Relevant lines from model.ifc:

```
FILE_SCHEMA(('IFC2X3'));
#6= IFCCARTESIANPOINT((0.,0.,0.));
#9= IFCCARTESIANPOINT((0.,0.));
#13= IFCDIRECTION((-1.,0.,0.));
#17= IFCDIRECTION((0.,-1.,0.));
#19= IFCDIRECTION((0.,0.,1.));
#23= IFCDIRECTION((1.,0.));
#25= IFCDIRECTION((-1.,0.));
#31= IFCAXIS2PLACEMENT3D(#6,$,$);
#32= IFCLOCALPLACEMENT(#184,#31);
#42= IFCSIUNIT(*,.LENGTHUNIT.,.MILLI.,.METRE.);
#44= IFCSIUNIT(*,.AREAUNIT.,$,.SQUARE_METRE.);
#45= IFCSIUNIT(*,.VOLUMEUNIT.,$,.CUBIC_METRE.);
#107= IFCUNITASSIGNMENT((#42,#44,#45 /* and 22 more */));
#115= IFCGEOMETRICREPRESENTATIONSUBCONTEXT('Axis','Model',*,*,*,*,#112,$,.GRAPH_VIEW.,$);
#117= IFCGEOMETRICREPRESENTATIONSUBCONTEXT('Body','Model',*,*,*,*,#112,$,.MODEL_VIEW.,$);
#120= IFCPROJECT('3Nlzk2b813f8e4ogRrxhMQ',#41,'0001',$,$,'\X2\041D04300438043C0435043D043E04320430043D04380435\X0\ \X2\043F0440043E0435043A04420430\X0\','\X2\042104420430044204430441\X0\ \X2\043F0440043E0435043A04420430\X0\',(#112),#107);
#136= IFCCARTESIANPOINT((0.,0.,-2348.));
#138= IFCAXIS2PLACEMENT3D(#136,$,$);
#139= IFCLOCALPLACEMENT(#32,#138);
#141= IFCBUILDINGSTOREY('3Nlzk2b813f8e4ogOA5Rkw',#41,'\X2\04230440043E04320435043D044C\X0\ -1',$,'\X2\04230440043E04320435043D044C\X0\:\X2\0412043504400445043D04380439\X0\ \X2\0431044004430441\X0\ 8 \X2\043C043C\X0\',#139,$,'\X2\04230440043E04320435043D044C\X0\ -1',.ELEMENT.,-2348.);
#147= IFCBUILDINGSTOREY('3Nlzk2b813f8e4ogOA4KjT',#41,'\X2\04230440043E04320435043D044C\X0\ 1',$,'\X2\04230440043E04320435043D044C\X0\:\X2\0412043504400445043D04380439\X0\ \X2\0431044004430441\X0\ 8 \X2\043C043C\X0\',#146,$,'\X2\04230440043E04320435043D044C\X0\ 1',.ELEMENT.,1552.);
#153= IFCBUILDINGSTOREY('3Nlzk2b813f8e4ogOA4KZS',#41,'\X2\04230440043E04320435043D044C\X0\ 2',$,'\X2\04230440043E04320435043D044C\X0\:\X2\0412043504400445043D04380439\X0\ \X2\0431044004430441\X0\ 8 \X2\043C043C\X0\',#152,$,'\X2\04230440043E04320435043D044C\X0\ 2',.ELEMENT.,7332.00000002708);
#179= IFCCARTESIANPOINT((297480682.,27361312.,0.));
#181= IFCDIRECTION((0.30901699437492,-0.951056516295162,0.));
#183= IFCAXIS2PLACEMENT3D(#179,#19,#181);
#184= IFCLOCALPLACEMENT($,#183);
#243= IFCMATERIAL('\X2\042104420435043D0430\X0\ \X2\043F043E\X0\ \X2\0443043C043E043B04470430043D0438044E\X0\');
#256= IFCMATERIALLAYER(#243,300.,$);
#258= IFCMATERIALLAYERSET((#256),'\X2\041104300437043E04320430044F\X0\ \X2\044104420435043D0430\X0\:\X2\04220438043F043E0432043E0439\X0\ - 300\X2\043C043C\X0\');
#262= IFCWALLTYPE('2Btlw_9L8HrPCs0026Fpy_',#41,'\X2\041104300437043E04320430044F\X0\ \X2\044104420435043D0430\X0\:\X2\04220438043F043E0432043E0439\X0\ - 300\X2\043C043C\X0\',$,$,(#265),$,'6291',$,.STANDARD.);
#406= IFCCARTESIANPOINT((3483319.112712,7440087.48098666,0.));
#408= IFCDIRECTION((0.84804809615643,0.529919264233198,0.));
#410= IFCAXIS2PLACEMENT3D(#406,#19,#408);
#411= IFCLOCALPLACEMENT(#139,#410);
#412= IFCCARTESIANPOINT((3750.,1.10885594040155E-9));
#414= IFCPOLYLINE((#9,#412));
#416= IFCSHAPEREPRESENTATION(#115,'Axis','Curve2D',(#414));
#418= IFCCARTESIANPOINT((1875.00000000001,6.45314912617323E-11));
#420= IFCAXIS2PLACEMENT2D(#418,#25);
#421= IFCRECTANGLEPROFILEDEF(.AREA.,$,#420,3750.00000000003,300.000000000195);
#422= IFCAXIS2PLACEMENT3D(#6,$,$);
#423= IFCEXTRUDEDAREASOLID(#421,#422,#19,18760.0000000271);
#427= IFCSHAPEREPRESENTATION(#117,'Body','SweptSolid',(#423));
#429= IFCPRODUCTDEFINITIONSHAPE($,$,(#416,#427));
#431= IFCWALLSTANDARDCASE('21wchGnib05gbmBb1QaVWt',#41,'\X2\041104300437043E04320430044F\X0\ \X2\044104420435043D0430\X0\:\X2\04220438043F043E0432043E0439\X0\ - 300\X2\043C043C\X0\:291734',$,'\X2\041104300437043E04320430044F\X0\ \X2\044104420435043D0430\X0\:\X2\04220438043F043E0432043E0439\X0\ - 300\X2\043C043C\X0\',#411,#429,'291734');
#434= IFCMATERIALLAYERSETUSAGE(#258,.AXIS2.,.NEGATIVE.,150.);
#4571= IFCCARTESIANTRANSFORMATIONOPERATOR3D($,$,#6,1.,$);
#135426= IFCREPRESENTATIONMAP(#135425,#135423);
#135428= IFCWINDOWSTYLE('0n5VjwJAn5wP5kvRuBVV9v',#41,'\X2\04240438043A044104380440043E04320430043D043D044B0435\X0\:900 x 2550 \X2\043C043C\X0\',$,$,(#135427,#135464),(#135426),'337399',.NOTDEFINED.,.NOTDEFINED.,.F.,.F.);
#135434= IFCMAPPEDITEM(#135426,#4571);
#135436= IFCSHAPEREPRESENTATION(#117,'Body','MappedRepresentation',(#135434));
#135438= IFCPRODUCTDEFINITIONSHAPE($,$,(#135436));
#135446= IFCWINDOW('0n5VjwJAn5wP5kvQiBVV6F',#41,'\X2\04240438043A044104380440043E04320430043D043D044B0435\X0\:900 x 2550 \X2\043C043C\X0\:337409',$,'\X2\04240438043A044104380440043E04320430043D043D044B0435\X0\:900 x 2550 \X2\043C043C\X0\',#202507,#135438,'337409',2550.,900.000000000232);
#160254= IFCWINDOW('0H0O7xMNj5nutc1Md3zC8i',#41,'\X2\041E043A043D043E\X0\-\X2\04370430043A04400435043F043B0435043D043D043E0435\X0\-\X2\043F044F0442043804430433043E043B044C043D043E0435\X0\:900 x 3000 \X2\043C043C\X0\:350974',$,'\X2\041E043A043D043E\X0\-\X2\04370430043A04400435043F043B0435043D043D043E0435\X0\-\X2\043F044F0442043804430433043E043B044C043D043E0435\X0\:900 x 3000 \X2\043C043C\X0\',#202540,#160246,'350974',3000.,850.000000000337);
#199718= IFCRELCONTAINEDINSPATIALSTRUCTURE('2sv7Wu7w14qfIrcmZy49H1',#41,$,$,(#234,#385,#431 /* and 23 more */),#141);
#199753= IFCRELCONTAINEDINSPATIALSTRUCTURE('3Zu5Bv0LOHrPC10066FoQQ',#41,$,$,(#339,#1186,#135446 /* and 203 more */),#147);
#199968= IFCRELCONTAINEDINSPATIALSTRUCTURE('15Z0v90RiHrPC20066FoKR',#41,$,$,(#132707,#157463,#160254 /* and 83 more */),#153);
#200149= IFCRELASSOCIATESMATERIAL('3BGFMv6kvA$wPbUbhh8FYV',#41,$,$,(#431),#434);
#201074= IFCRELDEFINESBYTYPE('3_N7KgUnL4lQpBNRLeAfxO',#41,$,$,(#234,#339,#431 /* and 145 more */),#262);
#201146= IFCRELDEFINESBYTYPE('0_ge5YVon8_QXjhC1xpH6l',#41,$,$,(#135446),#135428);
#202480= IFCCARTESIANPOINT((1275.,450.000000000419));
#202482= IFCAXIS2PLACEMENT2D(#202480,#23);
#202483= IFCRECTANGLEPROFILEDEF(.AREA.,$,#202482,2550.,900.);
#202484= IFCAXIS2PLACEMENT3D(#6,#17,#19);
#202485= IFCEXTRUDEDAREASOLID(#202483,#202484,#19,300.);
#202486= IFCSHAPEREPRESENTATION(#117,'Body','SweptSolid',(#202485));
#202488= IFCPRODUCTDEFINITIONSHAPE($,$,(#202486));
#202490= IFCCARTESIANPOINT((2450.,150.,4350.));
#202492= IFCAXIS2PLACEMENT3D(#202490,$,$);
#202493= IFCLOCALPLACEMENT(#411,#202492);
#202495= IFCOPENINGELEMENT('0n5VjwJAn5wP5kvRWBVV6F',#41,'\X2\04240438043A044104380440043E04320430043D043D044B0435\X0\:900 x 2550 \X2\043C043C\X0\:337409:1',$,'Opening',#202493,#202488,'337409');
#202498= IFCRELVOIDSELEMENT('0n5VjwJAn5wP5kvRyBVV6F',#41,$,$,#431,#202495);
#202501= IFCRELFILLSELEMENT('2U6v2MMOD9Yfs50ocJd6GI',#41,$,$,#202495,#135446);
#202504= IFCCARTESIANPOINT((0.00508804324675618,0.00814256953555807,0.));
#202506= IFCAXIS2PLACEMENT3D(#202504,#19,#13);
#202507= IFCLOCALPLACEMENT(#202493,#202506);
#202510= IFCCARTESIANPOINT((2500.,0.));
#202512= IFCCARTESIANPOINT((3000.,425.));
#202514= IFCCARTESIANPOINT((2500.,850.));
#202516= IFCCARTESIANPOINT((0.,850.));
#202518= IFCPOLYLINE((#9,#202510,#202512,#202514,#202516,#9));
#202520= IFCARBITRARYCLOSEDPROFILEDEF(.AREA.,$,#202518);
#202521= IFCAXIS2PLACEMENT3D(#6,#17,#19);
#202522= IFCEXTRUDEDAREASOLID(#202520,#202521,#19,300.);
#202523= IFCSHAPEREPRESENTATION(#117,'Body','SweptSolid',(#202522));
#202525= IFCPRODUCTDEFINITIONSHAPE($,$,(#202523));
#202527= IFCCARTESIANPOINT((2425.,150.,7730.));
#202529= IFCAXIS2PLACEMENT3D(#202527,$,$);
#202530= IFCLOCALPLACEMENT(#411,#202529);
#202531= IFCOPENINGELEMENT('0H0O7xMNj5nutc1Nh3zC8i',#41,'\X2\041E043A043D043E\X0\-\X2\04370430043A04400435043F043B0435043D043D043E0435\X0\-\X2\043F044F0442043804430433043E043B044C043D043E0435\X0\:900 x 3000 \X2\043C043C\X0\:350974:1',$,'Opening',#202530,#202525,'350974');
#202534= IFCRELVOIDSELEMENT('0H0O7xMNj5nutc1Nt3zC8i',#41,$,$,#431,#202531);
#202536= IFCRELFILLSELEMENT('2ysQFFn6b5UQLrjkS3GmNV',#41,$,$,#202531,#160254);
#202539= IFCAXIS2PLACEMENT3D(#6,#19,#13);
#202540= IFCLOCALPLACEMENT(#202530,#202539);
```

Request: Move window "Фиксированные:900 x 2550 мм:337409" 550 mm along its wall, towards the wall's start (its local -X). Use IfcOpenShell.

```python
import ifcopenshell
import ifcopenshell.api.geometry
import ifcopenshell.util.placement
import ifcopenshell.util.unit

model = ifcopenshell.open("model.ifc")
unit_scale = ifcopenshell.util.unit.calculate_unit_scale(model)

window = model.by_id(135446)
opening = window.FillsVoids[0].RelatingOpeningElement
wall = opening.VoidsElements[0].RelatingBuildingElement

wall_matrix = ifcopenshell.util.placement.get_local_placement(wall.ObjectPlacement)
shift = wall_matrix[:3, 0] * -0.55 / unit_scale
before = ifcopenshell.util.placement.get_local_placement(window.ObjectPlacement)[:3, 3].copy()

# The window is placed relative to its opening, so it follows when the opening moves.
matrix = ifcopenshell.util.placement.get_local_placement(opening.ObjectPlacement)
matrix[:3, 3] += shift
ifcopenshell.api.geometry.edit_object_placement(
    model, product=opening, matrix=matrix, is_si=False, should_transform_children=True
)

after = ifcopenshell.util.placement.get_local_placement(window.ObjectPlacement)[:3, 3]
print("window moved by", (after - before).round(3) + 0.0)

model.write("model_updated.ifc")
```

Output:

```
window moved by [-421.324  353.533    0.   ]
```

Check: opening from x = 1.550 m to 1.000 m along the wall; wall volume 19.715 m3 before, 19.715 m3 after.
